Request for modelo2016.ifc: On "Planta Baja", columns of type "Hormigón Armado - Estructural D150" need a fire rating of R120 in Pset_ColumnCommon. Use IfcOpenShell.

First a look at what the model holds.

```python
import ifcopenshell
import ifcopenshell.util.element

model = ifcopenshell.open("modelo2016.ifc")
print(model.schema)
storey = next(s for s in model.by_type("IfcBuildingStorey") if s.Name == "Planta Baja")
columns = [e for e in ifcopenshell.util.element.get_decomposition(storey) if e.is_a("IfcColumn")]
seen = {}
for e in columns:
    element_type = ifcopenshell.util.element.get_type(e)
    key = (element_type.Name if element_type != e and element_type else None, ifcopenshell.util.element.get_pset(e, "Pset_ColumnCommon", "FireRating"))
    seen[key] = seen.get(key, 0) + 1
for (name, value), count in sorted(seen.items(), key=str):
    print(count, "x", name, "|", value)
```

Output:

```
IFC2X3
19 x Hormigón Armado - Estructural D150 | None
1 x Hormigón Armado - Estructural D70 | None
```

```python
import ifcopenshell
import ifcopenshell.api.pset
import ifcopenshell.util.element

model = ifcopenshell.open("modelo2016.ifc")

storey = next(s for s in model.by_type("IfcBuildingStorey") if s.Name == "Planta Baja")
columns = [e for e in ifcopenshell.util.element.get_decomposition(storey) if e.is_a("IfcColumn")]

count = 0
for e in columns:
    element_type = ifcopenshell.util.element.get_type(e)
    if element_type in (None, e) or element_type.Name != "Hormigón Armado - Estructural D150":
        continue
    # add_pset returns the element's existing set when there is one.
    pset = ifcopenshell.api.pset.add_pset(model, product=e, name="Pset_ColumnCommon")
    ifcopenshell.api.pset.edit_pset(model, pset=pset, properties={"FireRating": "R120"})
    count += 1

print(count, "columns updated")

model.write("modelo2016_rev.ifc")
```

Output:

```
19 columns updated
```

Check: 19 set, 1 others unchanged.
